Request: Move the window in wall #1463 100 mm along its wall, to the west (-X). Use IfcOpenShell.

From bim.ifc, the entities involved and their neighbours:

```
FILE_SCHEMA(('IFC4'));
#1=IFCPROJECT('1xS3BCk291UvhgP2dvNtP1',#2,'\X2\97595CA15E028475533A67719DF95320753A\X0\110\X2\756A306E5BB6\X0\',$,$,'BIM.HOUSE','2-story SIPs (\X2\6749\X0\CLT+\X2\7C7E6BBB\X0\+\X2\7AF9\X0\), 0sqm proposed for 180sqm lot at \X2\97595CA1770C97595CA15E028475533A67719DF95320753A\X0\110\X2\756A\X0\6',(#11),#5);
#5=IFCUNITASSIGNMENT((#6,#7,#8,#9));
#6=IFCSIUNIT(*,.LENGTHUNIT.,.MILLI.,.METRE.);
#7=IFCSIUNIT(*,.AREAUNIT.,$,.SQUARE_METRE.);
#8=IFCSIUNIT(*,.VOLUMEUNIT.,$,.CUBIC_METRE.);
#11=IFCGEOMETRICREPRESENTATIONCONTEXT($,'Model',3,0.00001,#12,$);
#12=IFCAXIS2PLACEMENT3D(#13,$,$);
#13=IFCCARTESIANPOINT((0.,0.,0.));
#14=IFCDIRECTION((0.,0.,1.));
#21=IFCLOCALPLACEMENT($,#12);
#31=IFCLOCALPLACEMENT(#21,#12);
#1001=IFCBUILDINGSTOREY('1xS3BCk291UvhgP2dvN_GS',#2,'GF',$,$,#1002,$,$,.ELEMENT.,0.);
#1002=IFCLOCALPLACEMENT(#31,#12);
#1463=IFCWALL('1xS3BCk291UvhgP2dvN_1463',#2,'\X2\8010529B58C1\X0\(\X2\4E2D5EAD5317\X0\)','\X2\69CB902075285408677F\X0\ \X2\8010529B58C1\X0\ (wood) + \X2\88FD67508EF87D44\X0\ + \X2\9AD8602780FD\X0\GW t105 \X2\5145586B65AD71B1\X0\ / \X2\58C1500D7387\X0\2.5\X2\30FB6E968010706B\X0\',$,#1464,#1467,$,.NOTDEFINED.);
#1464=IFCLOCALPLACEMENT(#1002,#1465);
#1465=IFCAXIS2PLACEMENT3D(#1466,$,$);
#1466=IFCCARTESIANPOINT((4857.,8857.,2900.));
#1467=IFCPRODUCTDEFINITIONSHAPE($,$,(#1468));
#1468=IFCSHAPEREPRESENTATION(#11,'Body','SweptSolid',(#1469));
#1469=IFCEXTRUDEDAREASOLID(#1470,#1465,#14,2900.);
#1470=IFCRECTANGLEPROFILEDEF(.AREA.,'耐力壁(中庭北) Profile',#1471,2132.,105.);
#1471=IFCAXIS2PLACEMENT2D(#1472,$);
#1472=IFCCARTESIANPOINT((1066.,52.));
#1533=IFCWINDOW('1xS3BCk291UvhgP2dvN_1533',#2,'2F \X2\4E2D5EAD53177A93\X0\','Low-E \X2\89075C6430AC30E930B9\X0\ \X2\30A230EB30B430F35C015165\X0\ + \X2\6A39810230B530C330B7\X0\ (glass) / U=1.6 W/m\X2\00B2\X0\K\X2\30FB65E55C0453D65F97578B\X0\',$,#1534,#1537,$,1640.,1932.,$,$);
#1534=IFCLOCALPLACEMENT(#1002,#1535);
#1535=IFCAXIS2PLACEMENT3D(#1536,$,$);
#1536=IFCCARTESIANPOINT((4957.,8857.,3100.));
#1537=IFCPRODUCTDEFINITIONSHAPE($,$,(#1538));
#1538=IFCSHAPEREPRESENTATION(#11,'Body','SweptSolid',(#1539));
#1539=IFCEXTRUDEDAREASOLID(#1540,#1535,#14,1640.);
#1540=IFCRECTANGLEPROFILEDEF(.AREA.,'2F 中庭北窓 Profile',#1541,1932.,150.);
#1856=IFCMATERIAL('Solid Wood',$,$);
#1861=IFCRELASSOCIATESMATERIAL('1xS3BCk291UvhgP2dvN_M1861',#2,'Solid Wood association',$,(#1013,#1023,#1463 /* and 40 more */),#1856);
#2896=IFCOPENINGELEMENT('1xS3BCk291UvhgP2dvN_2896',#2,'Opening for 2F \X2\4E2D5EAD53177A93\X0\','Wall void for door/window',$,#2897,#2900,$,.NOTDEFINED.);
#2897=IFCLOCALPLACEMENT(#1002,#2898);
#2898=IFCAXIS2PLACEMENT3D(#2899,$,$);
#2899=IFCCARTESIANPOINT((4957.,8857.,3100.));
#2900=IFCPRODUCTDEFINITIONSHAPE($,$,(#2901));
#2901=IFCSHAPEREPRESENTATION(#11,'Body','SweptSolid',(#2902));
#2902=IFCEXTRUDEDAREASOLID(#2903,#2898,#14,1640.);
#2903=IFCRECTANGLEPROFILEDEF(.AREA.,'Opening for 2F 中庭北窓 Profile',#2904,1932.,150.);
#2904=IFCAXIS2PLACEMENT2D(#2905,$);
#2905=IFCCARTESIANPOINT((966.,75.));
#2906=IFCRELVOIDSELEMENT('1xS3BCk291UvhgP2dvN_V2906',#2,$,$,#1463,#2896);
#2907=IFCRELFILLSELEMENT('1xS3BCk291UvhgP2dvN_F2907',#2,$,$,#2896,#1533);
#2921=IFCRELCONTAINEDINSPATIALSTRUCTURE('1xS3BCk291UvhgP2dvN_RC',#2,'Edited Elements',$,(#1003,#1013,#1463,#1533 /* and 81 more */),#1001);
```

```python
import ifcopenshell
import ifcopenshell.api.geometry
import ifcopenshell.util.placement
import ifcopenshell.util.unit

model = ifcopenshell.open("bim.ifc")
unit_scale = ifcopenshell.util.unit.calculate_unit_scale(model)

window = model.by_guid("1xS3BCk291UvhgP2dvN_1533")
opening = window.FillsVoids[0].RelatingOpeningElement
wall = opening.VoidsElements[0].RelatingBuildingElement

wall_matrix = ifcopenshell.util.placement.get_local_placement(wall.ObjectPlacement)
shift = wall_matrix[:3, 0] * -0.1 / unit_scale
before = ifcopenshell.util.placement.get_local_placement(window.ObjectPlacement)[:3, 3].copy()

# The window is not placed relative to its opening, so move both.
for product in (opening, window):
    matrix = ifcopenshell.util.placement.get_local_placement(product.ObjectPlacement)
    matrix[:3, 3] += shift
    ifcopenshell.api.geometry.edit_object_placement(model, product=product, matrix=matrix, is_si=False)

after = ifcopenshell.util.placement.get_local_placement(window.ObjectPlacement)[:3, 3]
print("window moved by", (after - before).round(3) + 0.0)

model.write("bim_updated.ifc")
```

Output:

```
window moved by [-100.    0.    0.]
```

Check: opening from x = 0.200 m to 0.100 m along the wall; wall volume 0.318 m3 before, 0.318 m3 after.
